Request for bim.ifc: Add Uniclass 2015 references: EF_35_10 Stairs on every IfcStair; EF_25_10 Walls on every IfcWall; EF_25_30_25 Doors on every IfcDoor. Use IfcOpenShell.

First a look at what the model holds.

```python
import ifcopenshell

model = ifcopenshell.open("bim.ifc")
print(model.schema)
print("classifications:", [c.Name for c in model.by_type("IfcClassification")])
for ifc_class in ("IfcDoor", "IfcRoof", "IfcStair", "IfcWall", "IfcWindow"):
    print(ifc_class, len(model.by_type(ifc_class)))
```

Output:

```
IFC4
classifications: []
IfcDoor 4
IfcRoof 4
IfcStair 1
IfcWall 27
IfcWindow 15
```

```python
import ifcopenshell
import ifcopenshell.api.classification

model = ifcopenshell.open("bim.ifc")

system = ifcopenshell.api.classification.add_classification(model, classification="Uniclass 2015")

codes = {
    "IfcStair": ("EF_35_10", "Stairs"),
    "IfcWall": ("EF_25_10", "Walls"),
    "IfcDoor": ("EF_25_30_25", "Doors"),
}
for ifc_class, (code, name) in codes.items():
    products = model.by_type(ifc_class)
    ifcopenshell.api.classification.add_reference(
        model, products=products, classification=system, identification=code, name=name
    )
    print(code, len(products))

model.write("bim_edited.ifc")
```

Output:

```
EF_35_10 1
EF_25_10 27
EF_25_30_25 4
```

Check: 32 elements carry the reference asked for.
